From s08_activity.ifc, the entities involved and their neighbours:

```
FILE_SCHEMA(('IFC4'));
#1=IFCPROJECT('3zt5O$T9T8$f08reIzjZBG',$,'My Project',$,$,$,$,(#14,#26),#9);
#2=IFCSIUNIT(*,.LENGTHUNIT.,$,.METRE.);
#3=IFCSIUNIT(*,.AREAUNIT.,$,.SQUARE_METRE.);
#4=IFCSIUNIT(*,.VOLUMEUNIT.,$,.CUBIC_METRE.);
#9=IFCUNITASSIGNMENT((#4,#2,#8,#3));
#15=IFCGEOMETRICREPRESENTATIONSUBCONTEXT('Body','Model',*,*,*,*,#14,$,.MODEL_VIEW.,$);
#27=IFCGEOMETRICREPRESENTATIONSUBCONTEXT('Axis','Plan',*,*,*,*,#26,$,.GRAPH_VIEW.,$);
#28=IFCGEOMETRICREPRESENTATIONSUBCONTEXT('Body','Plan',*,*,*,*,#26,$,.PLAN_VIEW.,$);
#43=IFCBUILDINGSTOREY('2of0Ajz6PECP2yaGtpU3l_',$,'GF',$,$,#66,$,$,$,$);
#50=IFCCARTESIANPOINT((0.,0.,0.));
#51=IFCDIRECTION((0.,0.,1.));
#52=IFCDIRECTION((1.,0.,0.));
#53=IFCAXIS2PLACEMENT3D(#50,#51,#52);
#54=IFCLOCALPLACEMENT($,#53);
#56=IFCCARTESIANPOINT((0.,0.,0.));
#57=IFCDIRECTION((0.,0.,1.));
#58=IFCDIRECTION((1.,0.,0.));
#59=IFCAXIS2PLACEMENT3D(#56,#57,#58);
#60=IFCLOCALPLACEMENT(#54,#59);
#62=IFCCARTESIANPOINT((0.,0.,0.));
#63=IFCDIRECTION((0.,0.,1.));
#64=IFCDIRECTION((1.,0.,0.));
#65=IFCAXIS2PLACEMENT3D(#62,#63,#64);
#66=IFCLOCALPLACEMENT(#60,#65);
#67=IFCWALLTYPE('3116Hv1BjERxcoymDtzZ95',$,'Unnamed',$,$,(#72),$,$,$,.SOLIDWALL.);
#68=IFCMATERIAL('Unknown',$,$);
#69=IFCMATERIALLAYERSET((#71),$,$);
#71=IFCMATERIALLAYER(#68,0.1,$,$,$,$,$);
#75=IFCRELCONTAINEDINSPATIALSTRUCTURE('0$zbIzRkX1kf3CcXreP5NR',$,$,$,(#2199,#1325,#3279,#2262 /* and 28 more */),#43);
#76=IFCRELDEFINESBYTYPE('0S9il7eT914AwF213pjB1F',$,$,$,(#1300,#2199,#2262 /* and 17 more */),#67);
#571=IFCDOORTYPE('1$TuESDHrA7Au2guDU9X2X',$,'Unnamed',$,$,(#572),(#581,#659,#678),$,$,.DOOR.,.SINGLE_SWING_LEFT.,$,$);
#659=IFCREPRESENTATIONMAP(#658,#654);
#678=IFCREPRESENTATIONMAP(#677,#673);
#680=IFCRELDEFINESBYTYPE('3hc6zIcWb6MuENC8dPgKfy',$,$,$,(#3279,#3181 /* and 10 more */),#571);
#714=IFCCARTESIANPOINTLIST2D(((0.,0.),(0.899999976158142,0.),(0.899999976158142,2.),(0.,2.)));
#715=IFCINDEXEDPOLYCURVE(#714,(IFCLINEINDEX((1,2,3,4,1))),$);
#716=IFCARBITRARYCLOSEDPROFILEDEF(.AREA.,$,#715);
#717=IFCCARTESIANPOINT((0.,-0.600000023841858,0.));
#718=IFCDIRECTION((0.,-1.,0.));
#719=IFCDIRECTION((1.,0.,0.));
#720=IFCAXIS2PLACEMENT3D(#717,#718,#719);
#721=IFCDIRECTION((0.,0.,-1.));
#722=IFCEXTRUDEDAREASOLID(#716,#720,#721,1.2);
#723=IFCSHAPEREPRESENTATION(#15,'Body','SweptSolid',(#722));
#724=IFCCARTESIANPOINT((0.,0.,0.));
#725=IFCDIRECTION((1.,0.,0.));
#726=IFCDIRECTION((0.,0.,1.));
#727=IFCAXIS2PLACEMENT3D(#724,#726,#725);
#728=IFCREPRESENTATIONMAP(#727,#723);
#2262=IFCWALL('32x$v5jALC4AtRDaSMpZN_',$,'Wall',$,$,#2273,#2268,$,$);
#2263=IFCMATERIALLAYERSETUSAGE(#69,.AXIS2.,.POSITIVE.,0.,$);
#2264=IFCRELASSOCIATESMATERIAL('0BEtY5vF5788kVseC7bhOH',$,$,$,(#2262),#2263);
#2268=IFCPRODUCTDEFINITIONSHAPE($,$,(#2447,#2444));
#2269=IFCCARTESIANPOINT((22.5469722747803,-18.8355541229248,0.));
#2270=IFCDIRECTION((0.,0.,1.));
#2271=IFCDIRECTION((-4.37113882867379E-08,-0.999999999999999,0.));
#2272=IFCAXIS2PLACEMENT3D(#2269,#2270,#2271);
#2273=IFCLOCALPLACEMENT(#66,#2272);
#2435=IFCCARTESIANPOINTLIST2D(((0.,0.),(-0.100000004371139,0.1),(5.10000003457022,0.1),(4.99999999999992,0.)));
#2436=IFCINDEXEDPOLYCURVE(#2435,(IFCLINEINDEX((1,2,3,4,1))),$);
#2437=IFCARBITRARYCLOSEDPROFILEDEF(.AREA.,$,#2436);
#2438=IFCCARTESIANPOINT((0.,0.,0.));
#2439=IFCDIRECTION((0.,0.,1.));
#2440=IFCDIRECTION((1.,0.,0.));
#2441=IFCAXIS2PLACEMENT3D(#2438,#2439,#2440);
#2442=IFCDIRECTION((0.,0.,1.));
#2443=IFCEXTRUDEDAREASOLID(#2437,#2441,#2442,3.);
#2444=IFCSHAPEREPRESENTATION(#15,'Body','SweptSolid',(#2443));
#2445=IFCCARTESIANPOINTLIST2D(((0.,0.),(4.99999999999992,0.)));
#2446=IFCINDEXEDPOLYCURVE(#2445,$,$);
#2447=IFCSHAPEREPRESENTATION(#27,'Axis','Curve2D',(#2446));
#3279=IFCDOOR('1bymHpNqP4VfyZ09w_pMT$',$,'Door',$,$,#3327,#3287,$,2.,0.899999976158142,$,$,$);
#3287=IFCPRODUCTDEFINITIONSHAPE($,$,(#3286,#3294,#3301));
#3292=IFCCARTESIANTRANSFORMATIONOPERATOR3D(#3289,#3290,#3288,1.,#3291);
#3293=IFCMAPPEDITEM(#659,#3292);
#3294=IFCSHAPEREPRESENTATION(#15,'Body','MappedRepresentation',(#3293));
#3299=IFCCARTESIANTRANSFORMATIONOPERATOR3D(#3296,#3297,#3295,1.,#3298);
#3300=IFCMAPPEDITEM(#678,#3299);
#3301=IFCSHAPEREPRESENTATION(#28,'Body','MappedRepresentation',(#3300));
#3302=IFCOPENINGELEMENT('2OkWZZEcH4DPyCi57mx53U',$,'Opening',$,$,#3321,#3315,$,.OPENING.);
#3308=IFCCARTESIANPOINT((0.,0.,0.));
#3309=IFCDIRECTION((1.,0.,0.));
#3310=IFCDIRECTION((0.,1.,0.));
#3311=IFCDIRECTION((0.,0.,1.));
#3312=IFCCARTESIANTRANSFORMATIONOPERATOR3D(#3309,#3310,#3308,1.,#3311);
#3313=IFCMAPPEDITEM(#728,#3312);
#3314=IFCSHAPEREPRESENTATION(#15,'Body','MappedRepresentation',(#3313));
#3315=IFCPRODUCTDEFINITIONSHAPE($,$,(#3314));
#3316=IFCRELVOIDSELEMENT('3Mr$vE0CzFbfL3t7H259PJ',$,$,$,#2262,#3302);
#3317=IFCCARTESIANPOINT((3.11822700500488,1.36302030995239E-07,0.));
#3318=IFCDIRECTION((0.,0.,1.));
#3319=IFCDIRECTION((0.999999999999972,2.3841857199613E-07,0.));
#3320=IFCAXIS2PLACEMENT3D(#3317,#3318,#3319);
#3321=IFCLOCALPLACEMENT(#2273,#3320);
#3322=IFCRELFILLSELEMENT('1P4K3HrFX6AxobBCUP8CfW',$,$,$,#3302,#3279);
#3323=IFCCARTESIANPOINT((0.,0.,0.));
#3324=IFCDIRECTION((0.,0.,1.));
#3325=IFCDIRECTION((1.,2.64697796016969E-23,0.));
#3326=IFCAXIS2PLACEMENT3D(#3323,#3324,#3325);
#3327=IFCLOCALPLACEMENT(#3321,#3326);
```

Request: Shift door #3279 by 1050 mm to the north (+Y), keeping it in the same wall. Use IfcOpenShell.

```python
import ifcopenshell
import ifcopenshell.api.geometry
import ifcopenshell.util.placement
import ifcopenshell.util.unit

model = ifcopenshell.open("s08_activity.ifc")
unit_scale = ifcopenshell.util.unit.calculate_unit_scale(model)

door = model.by_guid("1bymHpNqP4VfyZ09w_pMT$")
opening = door.FillsVoids[0].RelatingOpeningElement
wall = opening.VoidsElements[0].RelatingBuildingElement

wall_matrix = ifcopenshell.util.placement.get_local_placement(wall.ObjectPlacement)
shift = wall_matrix[:3, 0] * -1.05 / unit_scale
before = ifcopenshell.util.placement.get_local_placement(door.ObjectPlacement)[:3, 3].copy()

# The door is placed relative to its opening, so it follows when the opening moves.
matrix = ifcopenshell.util.placement.get_local_placement(opening.ObjectPlacement)
matrix[:3, 3] += shift
ifcopenshell.api.geometry.edit_object_placement(
    model, product=opening, matrix=matrix, is_si=False, should_transform_children=True
)

after = ifcopenshell.util.placement.get_local_placement(door.ObjectPlacement)[:3, 3]
print("door moved by", (after - before).round(3) + 0.0)

model.write("s08_activity-out.ifc")
```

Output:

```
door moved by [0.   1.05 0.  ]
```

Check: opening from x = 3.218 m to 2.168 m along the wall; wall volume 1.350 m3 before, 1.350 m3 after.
